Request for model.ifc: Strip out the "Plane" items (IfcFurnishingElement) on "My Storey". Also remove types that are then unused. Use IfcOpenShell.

First a look at what the model holds.

```python
import ifcopenshell
import ifcopenshell.util.element

model = ifcopenshell.open("model.ifc")
print(model.schema)
storey = next(s for s in model.by_type("IfcBuildingStorey") if s.Name == "My Storey")
furniture = [e for e in ifcopenshell.util.element.get_decomposition(storey) if e.is_a("IfcFurnishingElement")]
seen = {}
for e in furniture:
    element_type = ifcopenshell.util.element.get_type(e)
    name = element_type.Name if element_type not in (None, e) else None
    seen[name] = seen.get(name, 0) + 1
for name, count in sorted(seen.items(), key=str):
    print(count, "x", name)
```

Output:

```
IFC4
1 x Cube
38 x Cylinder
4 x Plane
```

```python
import ifcopenshell
import ifcopenshell.api.root
import ifcopenshell.util.element

model = ifcopenshell.open("model.ifc")

storey = next(s for s in model.by_type("IfcBuildingStorey") if s.Name == "My Storey")
furniture = [e for e in ifcopenshell.util.element.get_decomposition(storey) if e.is_a("IfcFurnishingElement")]
targets = [e for e in furniture if (t := ifcopenshell.util.element.get_type(e)) not in (None, e) and t.Name == "Plane"]
types = {ifcopenshell.util.element.get_type(e) for e in targets} - {None, *targets}

for e in targets:
    ifcopenshell.api.root.remove_product(model, product=e)
print(len(targets), "removed")

unused = [t for t in types if not ifcopenshell.util.element.get_types(t)]
for t in unused:
    ifcopenshell.api.root.remove_product(model, product=t)
print(len(unused), "unused types removed")

model.write("model_updated.ifc")
```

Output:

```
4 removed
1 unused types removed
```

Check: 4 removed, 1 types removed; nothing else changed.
